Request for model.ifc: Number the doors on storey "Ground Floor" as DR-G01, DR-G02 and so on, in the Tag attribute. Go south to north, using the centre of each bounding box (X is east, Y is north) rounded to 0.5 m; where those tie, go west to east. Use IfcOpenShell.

First a look at what the model holds.

```python
import ifcopenshell
import ifcopenshell.util.element
import ifcopenshell.util.placement

model = ifcopenshell.open("model.ifc")
print(model.schema)
storey = next(s for s in model.by_type("IfcBuildingStorey") if s.Name == "Ground Floor")
doors = [e for e in ifcopenshell.util.element.get_decomposition(storey) if e.is_a("IfcDoor")]
for e in sorted(doors, key=lambda e: e.id()):
    origin = ifcopenshell.util.placement.get_local_placement(e.ObjectPlacement)[:3, 3]
    print(e.id(), e.Tag, e.Name, origin.round(2) + 0.0, sep=" | ")
```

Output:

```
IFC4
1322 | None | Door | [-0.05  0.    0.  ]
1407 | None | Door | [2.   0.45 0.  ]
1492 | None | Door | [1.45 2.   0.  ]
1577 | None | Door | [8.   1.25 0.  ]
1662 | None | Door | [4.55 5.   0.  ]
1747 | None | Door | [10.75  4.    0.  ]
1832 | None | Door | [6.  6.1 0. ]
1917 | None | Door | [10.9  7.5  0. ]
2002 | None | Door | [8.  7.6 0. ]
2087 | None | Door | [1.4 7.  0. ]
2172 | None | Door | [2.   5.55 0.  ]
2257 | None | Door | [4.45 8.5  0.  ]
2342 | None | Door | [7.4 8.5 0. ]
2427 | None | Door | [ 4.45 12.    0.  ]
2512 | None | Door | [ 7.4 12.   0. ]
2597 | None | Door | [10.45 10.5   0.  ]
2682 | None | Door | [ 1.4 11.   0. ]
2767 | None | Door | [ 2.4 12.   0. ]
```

```python
import ifcopenshell
import ifcopenshell.geom
import ifcopenshell.util.element
import ifcopenshell.util.shape

model = ifcopenshell.open("model.ifc")
settings = ifcopenshell.geom.settings()
settings.set("use-world-coords", True)


def centre(element):
    shape = ifcopenshell.geom.create_shape(settings, element)
    return ifcopenshell.util.shape.get_bbox_centroid(shape.geometry)


storey = next(s for s in model.by_type("IfcBuildingStorey") if s.Name == "Ground Floor")
doors = [e for e in ifcopenshell.util.element.get_decomposition(storey) if e.is_a("IfcDoor")]

# Insertion points can sit at a corner or the storey origin, so sort by the geometry (in metres).
centres = {e: centre(e) for e in doors}
doors.sort(key=lambda e: (round(centres[e][1] / 0.5), centres[e][0]))

for i, e in enumerate(doors, start=1):
    number = f"DR-G{i:02d}"
    e.Tag = number
    print(e.id(), number)

model.write("model_v2.ifc")
```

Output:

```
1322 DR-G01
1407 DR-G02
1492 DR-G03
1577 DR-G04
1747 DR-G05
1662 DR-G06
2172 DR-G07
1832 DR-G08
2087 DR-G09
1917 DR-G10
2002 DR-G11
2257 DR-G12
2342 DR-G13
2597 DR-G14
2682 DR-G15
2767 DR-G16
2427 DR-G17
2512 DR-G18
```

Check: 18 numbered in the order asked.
